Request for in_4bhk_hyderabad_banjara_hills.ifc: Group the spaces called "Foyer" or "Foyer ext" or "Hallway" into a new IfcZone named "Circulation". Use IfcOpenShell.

First a look at what the model holds.

```python
import ifcopenshell

model = ifcopenshell.open("in_4bhk_hyderabad_banjara_hills.ifc")
print(model.schema)
seen = {}
for space in model.by_type("IfcSpace"):
    seen[space.LongName] = seen.get(space.LongName, 0) + 1
for name, count in sorted(seen.items(), key=str):
    print(count, "x", name)
print("zones:", [z.Name for z in model.by_type("IfcZone")][:20])
```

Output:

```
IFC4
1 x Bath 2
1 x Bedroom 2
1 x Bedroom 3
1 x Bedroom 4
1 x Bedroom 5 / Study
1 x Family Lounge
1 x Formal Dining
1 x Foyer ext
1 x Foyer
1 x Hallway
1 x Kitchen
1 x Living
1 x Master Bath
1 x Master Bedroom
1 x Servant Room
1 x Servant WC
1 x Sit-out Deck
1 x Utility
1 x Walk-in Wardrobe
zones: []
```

```python
import ifcopenshell
import ifcopenshell.api.group
import ifcopenshell.api.root

model = ifcopenshell.open("in_4bhk_hyderabad_banjara_hills.ifc")

names = {"Foyer", "Foyer ext", "Hallway"}
spaces = [s for s in model.by_type("IfcSpace") if s.LongName in names]

zone = ifcopenshell.api.root.create_entity(model, ifc_class="IfcZone", name="Circulation")
ifcopenshell.api.group.assign_group(model, products=spaces, group=zone)
print(len(spaces), "spaces in", zone.Name)

model.write("in_4bhk_hyderabad_banjara_hills_rev.ifc")
```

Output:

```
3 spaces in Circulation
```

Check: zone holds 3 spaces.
